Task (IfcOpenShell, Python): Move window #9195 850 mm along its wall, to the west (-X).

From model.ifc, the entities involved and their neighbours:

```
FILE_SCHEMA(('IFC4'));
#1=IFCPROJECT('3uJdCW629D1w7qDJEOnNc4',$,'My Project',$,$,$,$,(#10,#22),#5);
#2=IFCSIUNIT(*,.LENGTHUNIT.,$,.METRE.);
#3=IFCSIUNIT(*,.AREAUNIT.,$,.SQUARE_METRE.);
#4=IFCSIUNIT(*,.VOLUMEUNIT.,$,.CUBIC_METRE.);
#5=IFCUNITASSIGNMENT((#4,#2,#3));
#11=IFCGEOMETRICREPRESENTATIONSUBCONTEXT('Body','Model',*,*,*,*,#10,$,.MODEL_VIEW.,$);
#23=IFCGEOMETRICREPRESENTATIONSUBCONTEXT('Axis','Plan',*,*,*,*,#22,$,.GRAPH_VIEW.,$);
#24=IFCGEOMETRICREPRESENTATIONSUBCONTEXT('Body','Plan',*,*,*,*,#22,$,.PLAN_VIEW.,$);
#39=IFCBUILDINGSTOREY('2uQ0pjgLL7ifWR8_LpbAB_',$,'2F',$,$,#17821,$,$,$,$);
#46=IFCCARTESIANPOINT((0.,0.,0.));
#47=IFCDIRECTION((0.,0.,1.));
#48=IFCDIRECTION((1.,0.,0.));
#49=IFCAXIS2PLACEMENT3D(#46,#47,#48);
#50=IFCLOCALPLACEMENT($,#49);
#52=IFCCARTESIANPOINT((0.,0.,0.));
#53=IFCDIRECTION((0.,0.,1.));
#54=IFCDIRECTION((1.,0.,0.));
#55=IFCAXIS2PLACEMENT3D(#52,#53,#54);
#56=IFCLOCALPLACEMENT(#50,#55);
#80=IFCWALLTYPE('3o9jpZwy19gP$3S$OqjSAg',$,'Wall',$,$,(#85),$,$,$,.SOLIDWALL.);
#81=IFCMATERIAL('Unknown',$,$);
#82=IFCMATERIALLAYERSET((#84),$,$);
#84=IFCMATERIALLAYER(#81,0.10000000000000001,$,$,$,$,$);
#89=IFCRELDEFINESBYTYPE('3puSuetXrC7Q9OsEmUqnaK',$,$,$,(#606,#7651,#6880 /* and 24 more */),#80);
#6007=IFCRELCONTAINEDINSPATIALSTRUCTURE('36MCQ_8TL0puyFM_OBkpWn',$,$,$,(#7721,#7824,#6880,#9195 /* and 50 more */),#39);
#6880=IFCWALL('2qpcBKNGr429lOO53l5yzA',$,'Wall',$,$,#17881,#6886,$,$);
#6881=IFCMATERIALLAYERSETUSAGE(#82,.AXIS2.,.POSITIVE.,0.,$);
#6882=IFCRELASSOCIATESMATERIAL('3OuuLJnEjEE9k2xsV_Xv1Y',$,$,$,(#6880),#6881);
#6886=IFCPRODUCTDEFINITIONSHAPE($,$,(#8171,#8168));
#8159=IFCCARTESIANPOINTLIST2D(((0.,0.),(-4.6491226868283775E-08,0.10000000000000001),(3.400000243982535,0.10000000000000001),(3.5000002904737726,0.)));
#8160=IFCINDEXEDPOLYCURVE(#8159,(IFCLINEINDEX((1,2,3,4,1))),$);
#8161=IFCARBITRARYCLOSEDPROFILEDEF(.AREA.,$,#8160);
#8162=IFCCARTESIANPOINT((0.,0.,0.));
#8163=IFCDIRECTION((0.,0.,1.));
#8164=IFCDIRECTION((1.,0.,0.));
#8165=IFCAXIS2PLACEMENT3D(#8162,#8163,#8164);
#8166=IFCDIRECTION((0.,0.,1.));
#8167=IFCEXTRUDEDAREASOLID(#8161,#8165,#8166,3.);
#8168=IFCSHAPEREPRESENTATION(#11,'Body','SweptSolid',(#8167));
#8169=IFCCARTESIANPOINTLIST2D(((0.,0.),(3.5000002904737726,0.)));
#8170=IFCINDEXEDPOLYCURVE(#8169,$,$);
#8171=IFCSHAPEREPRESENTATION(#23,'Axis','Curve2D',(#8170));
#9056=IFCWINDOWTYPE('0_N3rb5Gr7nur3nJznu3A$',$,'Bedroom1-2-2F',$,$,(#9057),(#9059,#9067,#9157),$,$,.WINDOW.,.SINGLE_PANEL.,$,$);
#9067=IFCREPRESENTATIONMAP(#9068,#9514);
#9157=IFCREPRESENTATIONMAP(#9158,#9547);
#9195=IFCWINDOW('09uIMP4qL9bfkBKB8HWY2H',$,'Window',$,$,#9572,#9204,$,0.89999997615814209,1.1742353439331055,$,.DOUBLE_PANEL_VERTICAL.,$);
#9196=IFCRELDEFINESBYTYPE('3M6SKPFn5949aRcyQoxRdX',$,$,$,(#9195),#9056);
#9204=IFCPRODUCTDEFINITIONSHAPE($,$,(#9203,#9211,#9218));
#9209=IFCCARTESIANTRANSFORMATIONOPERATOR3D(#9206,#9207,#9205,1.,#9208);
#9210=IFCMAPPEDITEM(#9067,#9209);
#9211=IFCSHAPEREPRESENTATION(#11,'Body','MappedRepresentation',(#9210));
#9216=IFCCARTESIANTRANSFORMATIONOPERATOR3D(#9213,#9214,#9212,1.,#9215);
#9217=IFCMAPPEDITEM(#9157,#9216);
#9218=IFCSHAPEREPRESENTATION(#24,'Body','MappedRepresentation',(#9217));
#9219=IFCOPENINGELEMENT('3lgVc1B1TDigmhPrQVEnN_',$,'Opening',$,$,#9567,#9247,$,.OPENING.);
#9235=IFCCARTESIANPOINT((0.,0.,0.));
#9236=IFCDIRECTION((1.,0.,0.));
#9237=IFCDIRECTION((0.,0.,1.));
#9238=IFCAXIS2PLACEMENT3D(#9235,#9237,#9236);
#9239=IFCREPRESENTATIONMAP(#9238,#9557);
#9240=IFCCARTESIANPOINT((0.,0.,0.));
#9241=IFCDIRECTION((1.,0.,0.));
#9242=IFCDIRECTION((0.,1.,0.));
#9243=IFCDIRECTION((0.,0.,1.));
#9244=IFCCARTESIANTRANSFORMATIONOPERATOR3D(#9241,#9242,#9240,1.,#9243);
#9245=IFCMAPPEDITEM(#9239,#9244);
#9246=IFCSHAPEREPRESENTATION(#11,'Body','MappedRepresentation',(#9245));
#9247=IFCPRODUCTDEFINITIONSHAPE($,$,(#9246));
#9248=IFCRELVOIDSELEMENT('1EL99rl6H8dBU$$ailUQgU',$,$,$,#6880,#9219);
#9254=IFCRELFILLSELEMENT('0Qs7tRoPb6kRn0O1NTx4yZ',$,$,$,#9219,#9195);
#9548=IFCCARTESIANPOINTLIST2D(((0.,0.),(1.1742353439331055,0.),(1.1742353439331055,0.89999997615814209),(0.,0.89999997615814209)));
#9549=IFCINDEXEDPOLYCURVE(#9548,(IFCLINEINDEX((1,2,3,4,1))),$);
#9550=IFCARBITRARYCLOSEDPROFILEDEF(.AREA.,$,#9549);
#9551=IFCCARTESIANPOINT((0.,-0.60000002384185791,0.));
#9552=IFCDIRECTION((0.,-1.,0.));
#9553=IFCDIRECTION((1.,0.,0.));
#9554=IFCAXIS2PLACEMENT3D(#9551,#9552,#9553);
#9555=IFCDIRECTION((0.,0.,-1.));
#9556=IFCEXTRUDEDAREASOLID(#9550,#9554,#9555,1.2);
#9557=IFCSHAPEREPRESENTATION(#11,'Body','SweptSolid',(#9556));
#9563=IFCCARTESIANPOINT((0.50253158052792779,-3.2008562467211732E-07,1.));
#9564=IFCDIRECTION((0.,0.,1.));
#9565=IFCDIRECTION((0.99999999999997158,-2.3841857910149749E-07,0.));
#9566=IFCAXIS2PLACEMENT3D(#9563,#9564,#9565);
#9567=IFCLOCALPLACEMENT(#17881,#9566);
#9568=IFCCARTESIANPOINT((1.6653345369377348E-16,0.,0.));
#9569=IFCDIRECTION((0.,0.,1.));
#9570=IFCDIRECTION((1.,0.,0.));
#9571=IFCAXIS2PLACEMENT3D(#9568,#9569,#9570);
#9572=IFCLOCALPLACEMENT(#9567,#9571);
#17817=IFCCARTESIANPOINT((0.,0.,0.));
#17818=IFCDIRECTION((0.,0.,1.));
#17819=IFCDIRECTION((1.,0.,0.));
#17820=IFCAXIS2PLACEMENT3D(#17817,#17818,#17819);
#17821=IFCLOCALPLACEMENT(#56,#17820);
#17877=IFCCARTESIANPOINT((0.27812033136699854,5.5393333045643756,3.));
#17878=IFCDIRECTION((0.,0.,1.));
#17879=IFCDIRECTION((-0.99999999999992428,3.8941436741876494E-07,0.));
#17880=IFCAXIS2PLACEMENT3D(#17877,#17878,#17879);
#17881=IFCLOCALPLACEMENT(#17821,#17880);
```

```python
import ifcopenshell
import ifcopenshell.api.geometry
import ifcopenshell.util.placement
import ifcopenshell.util.unit

model = ifcopenshell.open("model.ifc")
unit_scale = ifcopenshell.util.unit.calculate_unit_scale(model)

window = model.by_guid("09uIMP4qL9bfkBKB8HWY2H")
opening = window.FillsVoids[0].RelatingOpeningElement
wall = opening.VoidsElements[0].RelatingBuildingElement

wall_matrix = ifcopenshell.util.placement.get_local_placement(wall.ObjectPlacement)
shift = wall_matrix[:3, 0] * 0.85 / unit_scale
before = ifcopenshell.util.placement.get_local_placement(window.ObjectPlacement)[:3, 3].copy()

# The window is placed relative to its opening, so it follows when the opening moves.
matrix = ifcopenshell.util.placement.get_local_placement(opening.ObjectPlacement)
matrix[:3, 3] += shift
ifcopenshell.api.geometry.edit_object_placement(
    model, product=opening, matrix=matrix, is_si=False, should_transform_children=True
)

after = ifcopenshell.util.placement.get_local_placement(window.ObjectPlacement)[:3, 3]
print("window moved by", (after - before).round(3) + 0.0)

model.write("model_edited.ifc")
```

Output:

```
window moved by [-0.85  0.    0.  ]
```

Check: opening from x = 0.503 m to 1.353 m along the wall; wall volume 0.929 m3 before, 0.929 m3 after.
